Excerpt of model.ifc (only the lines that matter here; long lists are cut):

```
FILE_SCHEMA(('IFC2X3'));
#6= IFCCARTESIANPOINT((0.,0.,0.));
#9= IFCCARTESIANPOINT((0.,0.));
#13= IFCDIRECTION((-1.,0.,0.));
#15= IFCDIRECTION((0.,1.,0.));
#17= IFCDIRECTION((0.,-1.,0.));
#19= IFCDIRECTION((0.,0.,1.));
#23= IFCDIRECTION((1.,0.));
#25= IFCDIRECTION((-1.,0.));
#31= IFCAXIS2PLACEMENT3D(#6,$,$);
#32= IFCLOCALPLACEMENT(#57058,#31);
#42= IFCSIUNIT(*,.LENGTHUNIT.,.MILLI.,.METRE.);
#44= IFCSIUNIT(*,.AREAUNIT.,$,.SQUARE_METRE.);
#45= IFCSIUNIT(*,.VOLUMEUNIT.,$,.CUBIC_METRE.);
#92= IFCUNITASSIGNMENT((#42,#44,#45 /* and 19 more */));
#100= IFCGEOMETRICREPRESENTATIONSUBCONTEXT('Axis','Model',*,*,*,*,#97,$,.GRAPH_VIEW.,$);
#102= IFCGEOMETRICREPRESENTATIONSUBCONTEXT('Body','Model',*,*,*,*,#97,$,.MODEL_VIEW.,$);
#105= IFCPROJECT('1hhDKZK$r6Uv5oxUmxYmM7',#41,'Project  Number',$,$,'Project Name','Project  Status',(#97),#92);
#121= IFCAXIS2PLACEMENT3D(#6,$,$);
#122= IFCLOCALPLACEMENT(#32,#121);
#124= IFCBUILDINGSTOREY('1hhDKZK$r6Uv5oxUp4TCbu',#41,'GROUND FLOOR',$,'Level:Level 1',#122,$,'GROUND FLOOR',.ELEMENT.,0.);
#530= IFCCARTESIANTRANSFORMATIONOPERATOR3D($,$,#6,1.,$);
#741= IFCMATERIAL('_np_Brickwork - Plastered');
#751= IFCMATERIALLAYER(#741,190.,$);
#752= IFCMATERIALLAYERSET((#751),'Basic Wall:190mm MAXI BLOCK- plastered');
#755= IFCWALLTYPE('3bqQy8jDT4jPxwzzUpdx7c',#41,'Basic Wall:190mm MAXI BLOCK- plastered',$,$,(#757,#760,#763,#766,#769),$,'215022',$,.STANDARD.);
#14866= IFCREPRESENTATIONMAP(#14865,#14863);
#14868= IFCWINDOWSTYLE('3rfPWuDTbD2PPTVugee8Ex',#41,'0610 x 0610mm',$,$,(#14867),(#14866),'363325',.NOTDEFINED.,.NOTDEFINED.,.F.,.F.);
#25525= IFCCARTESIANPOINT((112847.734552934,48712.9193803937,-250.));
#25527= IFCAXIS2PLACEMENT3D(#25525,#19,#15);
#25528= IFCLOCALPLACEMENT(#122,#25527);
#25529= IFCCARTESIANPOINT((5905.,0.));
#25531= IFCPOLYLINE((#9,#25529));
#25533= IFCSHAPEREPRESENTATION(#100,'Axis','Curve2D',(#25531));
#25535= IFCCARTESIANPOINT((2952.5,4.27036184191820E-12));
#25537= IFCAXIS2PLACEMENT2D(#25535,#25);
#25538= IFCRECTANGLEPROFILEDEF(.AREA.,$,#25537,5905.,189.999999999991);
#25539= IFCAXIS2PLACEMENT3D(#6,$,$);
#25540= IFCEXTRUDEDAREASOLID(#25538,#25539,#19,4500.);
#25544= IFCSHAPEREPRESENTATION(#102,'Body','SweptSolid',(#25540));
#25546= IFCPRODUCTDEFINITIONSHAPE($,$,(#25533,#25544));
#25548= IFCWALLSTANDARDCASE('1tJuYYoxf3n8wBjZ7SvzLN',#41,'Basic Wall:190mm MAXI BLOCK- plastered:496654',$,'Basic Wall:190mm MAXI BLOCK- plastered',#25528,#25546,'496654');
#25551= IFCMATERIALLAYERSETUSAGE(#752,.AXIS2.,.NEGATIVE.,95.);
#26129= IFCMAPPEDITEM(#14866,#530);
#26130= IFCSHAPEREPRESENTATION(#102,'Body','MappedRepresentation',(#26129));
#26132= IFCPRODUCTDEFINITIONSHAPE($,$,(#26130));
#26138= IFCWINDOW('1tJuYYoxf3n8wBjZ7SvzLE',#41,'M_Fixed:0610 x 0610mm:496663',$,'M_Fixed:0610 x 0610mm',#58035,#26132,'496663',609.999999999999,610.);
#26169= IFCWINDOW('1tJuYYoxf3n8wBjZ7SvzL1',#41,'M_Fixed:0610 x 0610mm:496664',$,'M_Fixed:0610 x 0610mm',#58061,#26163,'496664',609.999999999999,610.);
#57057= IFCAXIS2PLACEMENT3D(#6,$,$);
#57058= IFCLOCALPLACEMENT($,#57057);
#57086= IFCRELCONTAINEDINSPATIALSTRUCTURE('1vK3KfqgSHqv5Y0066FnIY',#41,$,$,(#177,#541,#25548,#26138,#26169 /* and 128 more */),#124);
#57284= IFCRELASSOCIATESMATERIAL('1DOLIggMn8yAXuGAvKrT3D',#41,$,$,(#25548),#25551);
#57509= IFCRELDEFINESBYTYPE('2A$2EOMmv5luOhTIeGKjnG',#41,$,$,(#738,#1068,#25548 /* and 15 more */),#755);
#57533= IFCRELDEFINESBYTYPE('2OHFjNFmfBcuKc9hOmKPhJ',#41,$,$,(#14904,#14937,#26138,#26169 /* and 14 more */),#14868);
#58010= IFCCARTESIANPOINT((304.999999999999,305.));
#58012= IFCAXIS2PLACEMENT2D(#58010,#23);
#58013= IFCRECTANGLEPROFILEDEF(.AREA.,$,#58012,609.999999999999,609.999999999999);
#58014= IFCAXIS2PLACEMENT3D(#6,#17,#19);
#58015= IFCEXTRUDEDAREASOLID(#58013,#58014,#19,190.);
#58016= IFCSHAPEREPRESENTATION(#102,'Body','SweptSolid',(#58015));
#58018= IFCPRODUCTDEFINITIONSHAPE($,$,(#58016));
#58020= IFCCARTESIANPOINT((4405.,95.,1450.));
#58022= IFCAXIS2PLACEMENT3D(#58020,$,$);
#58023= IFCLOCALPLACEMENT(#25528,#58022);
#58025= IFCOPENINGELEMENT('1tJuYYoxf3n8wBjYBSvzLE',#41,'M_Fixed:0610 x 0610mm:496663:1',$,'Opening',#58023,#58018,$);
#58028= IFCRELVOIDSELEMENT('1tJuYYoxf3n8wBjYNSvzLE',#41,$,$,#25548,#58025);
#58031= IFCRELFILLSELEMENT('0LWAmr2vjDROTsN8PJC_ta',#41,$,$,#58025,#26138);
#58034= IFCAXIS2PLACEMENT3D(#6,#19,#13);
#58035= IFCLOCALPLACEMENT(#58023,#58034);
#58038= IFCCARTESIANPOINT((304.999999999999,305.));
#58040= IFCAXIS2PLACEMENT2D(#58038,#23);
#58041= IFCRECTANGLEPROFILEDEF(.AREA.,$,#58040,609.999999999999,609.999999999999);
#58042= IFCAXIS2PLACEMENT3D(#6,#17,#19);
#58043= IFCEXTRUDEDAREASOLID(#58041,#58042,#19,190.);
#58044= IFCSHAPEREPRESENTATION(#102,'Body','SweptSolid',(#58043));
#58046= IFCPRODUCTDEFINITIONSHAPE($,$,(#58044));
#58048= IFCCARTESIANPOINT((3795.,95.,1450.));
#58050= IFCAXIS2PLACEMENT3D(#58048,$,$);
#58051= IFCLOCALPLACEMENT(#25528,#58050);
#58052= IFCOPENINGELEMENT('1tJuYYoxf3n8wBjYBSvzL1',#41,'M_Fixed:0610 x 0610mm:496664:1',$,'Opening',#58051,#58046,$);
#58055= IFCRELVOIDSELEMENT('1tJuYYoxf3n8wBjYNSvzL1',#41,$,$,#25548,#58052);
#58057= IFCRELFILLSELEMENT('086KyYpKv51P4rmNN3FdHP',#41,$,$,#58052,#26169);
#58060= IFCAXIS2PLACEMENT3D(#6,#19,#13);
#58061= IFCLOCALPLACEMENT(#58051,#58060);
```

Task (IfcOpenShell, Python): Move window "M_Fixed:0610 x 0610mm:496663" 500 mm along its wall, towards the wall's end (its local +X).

```python
import ifcopenshell
import ifcopenshell.api.geometry
import ifcopenshell.util.placement

model = ifcopenshell.open("model.ifc")

window = model.by_guid("1tJuYYoxf3n8wBjZ7SvzLE")
opening = window.FillsVoids[0].RelatingOpeningElement
wall = opening.VoidsElements[0].RelatingBuildingElement

wall_matrix = ifcopenshell.util.placement.get_local_placement(wall.ObjectPlacement)
shift = wall_matrix[:3, 0] * 500.0
before = ifcopenshell.util.placement.get_local_placement(window.ObjectPlacement)[:3, 3].copy()

# The window is placed relative to its opening, so it follows when the opening moves.
matrix = ifcopenshell.util.placement.get_local_placement(opening.ObjectPlacement)
matrix[:3, 3] += shift
ifcopenshell.api.geometry.edit_object_placement(
    model, product=opening, matrix=matrix, is_si=False, should_transform_children=True
)

after = ifcopenshell.util.placement.get_local_placement(window.ObjectPlacement)[:3, 3]
print("window moved by", (after - before).round(3) + 0.0)

model.write("model_edited.ifc")
```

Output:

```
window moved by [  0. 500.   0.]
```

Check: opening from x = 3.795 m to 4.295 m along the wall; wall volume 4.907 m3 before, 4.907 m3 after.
